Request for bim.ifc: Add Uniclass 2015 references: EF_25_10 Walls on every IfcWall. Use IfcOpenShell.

First a look at what the model holds.

```python
import ifcopenshell

model = ifcopenshell.open("bim.ifc")
print(model.schema)
print("classifications:", [c.Name for c in model.by_type("IfcClassification")])
for ifc_class in ("IfcDoor", "IfcRoof", "IfcStair", "IfcWall", "IfcWindow"):
    print(ifc_class, len(model.by_type(ifc_class)))
```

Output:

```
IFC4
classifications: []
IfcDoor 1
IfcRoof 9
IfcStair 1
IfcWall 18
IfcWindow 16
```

```python
import ifcopenshell
import ifcopenshell.api.classification

model = ifcopenshell.open("bim.ifc")

system = ifcopenshell.api.classification.add_classification(model, classification="Uniclass 2015")

codes = {
    "IfcWall": ("EF_25_10", "Walls"),
}
for ifc_class, (code, name) in codes.items():
    products = model.by_type(ifc_class)
    ifcopenshell.api.classification.add_reference(
        model, products=products, classification=system, identification=code, name=name
    )
    print(code, len(products))

model.write("bim_v2.ifc")
```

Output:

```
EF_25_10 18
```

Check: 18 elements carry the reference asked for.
